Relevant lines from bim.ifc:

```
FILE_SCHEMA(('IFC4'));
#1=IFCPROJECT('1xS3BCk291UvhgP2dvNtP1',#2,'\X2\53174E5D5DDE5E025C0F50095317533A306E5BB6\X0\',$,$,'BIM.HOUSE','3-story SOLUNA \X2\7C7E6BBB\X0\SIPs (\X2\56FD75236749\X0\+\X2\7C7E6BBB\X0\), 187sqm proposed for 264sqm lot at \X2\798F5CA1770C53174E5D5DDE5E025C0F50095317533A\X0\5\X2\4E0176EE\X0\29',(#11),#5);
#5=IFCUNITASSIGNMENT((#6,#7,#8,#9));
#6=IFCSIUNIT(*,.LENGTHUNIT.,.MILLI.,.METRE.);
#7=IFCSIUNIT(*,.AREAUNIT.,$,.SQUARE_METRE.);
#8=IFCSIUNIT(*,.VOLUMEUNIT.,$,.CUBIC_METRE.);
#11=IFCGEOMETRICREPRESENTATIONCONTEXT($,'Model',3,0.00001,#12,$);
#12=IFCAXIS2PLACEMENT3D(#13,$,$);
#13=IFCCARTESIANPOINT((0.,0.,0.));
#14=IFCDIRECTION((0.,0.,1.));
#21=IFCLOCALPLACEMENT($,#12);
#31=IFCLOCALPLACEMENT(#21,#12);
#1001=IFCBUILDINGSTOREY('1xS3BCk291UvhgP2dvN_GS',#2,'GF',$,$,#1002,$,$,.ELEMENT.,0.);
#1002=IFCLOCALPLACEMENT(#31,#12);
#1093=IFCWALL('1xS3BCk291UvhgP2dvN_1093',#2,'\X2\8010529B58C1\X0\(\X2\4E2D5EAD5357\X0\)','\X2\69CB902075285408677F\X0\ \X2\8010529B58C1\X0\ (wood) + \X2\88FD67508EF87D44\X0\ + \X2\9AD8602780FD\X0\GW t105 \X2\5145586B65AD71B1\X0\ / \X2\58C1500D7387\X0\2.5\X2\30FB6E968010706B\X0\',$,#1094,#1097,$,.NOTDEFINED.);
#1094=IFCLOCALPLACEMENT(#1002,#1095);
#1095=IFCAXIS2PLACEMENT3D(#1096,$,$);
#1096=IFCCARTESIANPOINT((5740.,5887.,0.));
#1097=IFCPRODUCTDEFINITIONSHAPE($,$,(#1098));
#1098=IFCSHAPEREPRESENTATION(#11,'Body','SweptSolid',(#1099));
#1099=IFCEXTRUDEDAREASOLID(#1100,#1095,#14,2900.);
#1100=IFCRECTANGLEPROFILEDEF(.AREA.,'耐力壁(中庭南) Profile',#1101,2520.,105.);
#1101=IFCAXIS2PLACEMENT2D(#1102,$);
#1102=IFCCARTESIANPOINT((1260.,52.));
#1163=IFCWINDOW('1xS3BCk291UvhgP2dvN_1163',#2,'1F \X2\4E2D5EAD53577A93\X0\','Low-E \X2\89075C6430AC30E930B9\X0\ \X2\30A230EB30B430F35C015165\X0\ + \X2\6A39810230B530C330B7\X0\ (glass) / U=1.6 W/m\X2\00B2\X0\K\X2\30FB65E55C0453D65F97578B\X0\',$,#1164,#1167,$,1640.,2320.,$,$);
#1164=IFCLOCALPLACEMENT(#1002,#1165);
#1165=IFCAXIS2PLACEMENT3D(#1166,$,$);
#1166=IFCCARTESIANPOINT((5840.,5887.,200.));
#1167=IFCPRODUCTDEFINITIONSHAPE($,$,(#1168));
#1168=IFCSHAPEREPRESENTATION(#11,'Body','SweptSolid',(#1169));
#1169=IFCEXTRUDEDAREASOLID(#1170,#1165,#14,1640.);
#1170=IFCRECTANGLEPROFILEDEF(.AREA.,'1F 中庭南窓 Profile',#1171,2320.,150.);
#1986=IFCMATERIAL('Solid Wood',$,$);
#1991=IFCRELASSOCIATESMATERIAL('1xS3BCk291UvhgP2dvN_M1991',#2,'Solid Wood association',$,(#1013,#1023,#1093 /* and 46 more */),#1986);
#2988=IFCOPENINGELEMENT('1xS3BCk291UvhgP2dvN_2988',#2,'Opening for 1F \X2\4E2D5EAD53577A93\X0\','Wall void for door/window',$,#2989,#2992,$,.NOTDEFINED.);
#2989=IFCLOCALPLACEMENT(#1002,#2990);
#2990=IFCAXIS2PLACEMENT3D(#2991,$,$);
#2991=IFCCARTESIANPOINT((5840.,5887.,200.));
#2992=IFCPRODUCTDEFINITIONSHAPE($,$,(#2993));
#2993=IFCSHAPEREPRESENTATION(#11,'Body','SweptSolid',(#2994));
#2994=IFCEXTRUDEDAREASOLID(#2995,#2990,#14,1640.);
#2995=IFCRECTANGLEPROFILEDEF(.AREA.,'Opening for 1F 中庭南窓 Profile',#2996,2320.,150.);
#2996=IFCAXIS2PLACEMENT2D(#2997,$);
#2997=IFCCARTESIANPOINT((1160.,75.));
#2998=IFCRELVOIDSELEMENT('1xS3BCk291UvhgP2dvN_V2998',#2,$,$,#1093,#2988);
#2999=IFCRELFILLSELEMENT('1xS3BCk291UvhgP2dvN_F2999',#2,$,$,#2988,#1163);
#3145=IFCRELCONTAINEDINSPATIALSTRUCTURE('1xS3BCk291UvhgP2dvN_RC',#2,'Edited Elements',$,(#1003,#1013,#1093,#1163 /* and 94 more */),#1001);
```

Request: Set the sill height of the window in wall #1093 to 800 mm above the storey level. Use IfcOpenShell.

```python
import numpy as np
import ifcopenshell
import ifcopenshell.api.geometry
import ifcopenshell.geom
import ifcopenshell.util.element
import ifcopenshell.util.placement
import ifcopenshell.util.shape
import ifcopenshell.util.unit

model = ifcopenshell.open("bim.ifc")
unit_scale = ifcopenshell.util.unit.calculate_unit_scale(model)

window = model.by_guid("1xS3BCk291UvhgP2dvN_1163")
opening = window.FillsVoids[0].RelatingOpeningElement
storey = ifcopenshell.util.element.get_container(window, ifc_class="IfcBuildingStorey")
level = ifcopenshell.util.placement.get_local_placement(storey.ObjectPlacement)[2, 3]

# The opening's origin need not be at the sill, so measure its lowest point.
shape = ifcopenshell.geom.create_shape(ifcopenshell.geom.settings(), opening)
bottom = ifcopenshell.util.shape.get_shape_bottom_elevation(shape, shape.geometry) / unit_scale
dz = level + 800.0 - bottom

shift = np.array([0.0, 0.0, dz])
# The window is not placed relative to its opening, so move both.
for product in (opening, window):
    matrix = ifcopenshell.util.placement.get_local_placement(product.ObjectPlacement)
    matrix[:3, 3] += shift
    ifcopenshell.api.geometry.edit_object_placement(model, product=product, matrix=matrix, is_si=False)

print(f"moved by {dz * unit_scale:+.3f} m")

model.write("bim_updated.ifc")
```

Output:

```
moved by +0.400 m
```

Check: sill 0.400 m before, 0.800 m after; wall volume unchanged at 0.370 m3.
